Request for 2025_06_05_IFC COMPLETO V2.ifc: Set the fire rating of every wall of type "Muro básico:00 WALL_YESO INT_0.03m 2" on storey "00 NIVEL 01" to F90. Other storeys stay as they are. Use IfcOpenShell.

First a look at what the model holds.

```python
import ifcopenshell
import ifcopenshell.util.element

model = ifcopenshell.open("2025_06_05_IFC COMPLETO V2.ifc")
print(model.schema)
storey = next(s for s in model.by_type("IfcBuildingStorey") if s.Name == "00 NIVEL 01")
walls = [e for e in ifcopenshell.util.element.get_decomposition(storey) if e.is_a("IfcWall")]
seen = {}
for e in walls:
    element_type = ifcopenshell.util.element.get_type(e)
    key = (element_type.Name if element_type != e and element_type else None, ifcopenshell.util.element.get_pset(e, "Pset_WallCommon", "FireRating"))
    seen[key] = seen.get(key, 0) + 1
for (name, value), count in sorted(seen.items(), key=str):
    print(count, "x", name, "|", value)
```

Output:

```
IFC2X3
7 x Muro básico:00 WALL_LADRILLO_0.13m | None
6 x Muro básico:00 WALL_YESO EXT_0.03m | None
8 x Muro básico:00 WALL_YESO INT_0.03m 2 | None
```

```python
import ifcopenshell
import ifcopenshell.api.pset
import ifcopenshell.util.element

model = ifcopenshell.open("2025_06_05_IFC COMPLETO V2.ifc")

storey = next(s for s in model.by_type("IfcBuildingStorey") if s.Name == "00 NIVEL 01")
walls = [e for e in ifcopenshell.util.element.get_decomposition(storey) if e.is_a("IfcWall")]

count = 0
for e in walls:
    element_type = ifcopenshell.util.element.get_type(e)
    if element_type in (None, e) or element_type.Name != "Muro básico:00 WALL_YESO INT_0.03m 2":
        continue
    # add_pset returns the element's existing set when there is one.
    pset = ifcopenshell.api.pset.add_pset(model, product=e, name="Pset_WallCommon")
    ifcopenshell.api.pset.edit_pset(model, pset=pset, properties={"FireRating": "F90"})
    count += 1

print(count, "walls updated")

model.write("2025_06_05_IFC COMPLETO V2-out.ifc")
```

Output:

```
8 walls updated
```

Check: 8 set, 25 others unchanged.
